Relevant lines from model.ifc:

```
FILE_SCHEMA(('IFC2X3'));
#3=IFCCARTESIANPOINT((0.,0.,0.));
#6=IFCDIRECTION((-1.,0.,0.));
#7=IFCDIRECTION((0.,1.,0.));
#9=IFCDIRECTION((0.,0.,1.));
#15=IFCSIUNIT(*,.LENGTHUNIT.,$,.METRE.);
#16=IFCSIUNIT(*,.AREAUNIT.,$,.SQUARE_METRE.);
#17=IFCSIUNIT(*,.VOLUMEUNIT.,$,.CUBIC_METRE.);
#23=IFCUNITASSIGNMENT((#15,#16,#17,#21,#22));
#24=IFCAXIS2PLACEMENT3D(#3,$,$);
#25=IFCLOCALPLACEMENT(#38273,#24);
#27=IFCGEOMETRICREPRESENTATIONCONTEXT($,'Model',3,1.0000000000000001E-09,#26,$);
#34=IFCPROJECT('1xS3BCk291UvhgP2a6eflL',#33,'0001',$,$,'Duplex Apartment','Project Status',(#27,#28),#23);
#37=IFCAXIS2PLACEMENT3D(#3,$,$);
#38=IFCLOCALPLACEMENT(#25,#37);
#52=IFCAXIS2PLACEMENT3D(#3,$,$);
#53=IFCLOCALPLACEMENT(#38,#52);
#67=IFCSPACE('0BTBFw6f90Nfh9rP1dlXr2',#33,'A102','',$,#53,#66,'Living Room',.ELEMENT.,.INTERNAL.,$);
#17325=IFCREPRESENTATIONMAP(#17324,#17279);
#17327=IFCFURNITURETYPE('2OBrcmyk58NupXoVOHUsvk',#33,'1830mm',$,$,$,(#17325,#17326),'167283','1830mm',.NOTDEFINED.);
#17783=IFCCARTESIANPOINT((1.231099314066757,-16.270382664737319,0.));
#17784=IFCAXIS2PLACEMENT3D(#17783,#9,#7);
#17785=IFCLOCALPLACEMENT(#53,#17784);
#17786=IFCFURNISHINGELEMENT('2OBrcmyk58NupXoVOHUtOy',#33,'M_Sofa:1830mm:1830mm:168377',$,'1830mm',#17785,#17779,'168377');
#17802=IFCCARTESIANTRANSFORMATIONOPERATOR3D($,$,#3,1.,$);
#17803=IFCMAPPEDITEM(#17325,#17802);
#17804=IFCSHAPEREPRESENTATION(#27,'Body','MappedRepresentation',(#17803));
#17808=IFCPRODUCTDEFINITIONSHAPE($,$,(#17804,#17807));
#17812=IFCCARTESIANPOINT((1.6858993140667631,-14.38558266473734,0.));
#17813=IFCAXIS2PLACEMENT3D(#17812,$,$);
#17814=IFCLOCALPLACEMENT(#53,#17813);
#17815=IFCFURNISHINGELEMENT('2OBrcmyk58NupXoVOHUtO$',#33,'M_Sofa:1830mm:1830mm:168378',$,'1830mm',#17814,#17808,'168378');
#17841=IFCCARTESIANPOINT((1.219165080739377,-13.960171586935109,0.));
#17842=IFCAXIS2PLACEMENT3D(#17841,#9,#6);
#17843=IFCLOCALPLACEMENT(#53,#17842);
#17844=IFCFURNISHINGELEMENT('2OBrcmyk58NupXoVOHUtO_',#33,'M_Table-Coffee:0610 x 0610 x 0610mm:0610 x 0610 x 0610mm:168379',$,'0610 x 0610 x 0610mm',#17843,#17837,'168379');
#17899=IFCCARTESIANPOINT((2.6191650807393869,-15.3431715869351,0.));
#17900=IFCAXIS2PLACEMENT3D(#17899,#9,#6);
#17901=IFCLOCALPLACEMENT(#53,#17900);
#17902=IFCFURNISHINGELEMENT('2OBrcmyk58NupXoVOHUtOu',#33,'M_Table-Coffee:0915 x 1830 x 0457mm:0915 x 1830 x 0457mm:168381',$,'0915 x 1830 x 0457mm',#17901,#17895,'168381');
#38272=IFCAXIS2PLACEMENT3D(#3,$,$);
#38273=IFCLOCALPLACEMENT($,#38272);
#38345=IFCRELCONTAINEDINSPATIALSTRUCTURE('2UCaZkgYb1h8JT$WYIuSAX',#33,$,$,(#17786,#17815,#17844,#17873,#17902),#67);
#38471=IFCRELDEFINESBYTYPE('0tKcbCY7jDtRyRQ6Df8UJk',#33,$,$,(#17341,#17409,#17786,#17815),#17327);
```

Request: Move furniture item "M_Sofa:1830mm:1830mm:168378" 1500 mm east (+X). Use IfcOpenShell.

```python
import ifcopenshell
import ifcopenshell.api.geometry
import ifcopenshell.util.placement

model = ifcopenshell.open("model.ifc")

item = model.by_id(17815)
matrix = ifcopenshell.util.placement.get_local_placement(item.ObjectPlacement)
matrix[0, 3] += 1.5
ifcopenshell.api.geometry.edit_object_placement(model, product=item, matrix=matrix, is_si=False)

print(ifcopenshell.util.placement.get_local_placement(item.ObjectPlacement).round(3) + 0.0)

model.write("model-out.ifc")
```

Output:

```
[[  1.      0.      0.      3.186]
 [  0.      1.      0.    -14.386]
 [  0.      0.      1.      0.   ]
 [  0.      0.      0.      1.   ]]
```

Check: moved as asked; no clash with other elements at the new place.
